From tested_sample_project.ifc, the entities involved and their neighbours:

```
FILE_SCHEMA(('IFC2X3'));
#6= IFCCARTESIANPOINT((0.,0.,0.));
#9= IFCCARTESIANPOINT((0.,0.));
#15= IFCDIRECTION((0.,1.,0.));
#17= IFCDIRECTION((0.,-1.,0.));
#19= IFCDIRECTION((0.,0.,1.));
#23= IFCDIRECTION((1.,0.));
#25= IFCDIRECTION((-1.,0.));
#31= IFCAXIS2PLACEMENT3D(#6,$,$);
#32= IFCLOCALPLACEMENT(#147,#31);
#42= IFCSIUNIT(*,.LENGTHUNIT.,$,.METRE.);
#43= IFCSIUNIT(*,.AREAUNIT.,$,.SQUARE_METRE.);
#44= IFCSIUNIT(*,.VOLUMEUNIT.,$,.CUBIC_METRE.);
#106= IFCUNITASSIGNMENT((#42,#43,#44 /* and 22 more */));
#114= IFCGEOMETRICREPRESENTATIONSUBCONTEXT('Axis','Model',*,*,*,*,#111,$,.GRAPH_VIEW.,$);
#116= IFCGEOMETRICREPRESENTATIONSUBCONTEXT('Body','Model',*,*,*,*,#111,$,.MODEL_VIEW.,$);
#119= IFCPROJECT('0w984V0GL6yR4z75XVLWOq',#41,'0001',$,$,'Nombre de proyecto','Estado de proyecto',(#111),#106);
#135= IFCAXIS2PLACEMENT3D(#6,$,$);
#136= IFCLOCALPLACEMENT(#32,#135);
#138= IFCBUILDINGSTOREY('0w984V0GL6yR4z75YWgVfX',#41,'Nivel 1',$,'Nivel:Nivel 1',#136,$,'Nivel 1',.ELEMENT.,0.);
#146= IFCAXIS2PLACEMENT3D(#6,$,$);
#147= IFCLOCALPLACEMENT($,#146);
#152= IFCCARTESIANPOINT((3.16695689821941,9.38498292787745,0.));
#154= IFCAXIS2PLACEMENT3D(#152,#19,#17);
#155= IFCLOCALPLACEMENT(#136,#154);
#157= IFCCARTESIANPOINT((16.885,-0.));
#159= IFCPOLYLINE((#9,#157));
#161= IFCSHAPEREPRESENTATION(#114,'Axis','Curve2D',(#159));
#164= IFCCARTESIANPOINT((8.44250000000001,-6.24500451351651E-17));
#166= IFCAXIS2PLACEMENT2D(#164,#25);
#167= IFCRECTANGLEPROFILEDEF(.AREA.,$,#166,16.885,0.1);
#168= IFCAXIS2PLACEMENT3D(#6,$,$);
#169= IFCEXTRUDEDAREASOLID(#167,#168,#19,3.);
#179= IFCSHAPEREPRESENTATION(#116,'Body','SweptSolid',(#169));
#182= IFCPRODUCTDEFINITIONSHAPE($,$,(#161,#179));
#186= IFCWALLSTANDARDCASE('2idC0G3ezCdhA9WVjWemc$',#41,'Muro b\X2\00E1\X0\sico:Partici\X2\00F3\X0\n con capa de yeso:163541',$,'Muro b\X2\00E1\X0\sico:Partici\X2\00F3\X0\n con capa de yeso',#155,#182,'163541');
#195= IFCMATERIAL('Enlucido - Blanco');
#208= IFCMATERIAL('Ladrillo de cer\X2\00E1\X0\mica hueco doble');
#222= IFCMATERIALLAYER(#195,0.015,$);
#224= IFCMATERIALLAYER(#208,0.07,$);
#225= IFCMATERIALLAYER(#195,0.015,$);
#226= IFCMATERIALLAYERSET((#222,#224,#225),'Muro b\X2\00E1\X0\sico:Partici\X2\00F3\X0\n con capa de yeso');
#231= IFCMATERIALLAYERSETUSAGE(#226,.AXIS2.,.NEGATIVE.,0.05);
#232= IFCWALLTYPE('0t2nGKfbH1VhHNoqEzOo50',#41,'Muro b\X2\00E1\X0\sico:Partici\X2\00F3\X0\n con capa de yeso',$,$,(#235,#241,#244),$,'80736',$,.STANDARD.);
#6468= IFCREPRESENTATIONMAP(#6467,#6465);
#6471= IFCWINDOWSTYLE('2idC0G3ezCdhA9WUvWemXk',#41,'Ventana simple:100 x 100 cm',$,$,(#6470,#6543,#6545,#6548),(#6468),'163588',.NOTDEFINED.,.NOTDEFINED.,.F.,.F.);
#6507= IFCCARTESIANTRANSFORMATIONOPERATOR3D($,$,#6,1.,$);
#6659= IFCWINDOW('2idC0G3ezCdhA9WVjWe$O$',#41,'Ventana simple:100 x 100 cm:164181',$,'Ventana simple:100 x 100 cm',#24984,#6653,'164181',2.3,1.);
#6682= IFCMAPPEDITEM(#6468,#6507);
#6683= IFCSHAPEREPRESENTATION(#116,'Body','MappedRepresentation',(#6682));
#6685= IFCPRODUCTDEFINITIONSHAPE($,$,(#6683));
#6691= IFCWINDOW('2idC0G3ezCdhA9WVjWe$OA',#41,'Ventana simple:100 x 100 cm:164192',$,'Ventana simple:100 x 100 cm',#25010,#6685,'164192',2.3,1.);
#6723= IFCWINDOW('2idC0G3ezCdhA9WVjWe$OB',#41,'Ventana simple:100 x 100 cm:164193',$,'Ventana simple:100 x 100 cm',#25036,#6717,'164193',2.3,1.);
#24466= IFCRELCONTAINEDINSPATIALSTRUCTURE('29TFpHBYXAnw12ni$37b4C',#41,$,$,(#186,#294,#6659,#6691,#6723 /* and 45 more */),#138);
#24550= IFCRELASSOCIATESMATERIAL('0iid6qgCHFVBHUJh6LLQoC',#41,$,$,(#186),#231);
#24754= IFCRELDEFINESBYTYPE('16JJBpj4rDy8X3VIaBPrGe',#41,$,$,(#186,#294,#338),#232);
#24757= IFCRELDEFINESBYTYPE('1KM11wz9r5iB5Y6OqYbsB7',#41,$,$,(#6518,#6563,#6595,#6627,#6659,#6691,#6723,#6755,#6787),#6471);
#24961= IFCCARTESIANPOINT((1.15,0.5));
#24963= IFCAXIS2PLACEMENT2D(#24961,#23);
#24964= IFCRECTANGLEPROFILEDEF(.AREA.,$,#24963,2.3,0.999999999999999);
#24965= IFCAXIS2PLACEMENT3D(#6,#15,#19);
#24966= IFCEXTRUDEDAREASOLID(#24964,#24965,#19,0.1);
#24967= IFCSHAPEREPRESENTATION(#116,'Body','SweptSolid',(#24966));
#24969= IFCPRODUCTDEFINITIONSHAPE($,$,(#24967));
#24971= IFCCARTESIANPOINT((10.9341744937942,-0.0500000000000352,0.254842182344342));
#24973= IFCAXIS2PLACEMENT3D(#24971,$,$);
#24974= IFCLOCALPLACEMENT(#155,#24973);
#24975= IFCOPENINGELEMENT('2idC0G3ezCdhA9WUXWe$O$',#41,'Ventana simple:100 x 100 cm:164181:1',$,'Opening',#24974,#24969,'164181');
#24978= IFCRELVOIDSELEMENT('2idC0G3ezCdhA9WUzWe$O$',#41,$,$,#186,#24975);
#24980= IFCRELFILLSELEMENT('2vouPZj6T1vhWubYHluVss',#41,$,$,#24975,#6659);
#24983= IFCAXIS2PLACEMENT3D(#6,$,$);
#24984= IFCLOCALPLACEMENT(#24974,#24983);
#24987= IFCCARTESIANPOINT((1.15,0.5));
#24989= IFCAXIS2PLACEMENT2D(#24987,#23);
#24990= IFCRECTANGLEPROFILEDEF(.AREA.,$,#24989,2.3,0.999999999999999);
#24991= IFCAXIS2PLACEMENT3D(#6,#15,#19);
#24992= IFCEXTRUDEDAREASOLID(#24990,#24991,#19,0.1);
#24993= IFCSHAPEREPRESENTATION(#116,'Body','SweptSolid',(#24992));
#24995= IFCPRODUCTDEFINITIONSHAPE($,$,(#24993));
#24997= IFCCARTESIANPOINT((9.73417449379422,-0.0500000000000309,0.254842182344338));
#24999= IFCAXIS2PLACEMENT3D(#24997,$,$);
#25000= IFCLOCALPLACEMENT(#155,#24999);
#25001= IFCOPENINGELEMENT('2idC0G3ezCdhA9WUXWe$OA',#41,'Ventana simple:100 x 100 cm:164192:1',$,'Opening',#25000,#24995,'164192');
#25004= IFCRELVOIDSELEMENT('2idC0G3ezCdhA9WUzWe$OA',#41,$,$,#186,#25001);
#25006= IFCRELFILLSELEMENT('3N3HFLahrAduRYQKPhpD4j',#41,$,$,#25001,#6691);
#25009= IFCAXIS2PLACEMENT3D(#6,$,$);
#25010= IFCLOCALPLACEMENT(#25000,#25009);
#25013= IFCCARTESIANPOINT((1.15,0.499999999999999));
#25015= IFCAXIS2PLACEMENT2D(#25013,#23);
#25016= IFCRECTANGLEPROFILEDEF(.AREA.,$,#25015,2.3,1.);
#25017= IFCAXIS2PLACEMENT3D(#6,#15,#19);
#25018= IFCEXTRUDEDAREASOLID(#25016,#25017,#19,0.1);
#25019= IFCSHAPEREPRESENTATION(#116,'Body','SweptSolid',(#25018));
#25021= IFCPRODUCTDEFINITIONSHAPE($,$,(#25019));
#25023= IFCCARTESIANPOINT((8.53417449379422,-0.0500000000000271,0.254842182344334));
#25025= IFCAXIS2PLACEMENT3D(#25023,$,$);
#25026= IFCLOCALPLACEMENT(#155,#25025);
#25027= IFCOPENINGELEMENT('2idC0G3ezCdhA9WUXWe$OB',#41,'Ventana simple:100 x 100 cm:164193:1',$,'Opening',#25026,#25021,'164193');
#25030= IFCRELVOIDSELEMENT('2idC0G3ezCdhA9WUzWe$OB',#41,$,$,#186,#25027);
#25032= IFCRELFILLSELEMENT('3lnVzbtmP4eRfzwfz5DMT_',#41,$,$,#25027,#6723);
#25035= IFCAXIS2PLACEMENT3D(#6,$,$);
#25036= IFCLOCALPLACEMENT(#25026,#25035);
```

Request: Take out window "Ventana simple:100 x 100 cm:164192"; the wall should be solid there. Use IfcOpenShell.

```python
import ifcopenshell
import ifcopenshell.api.feature
import ifcopenshell.api.root
import ifcopenshell.geom
import ifcopenshell.util.shape

model = ifcopenshell.open("tested_sample_project.ifc")
settings = ifcopenshell.geom.settings()


def volume(element):
    """Net volume in cubic metres, openings subtracted."""
    shape = ifcopenshell.geom.create_shape(settings, element)
    return ifcopenshell.util.shape.get_volume(shape.geometry)


window = model.by_guid("2idC0G3ezCdhA9WVjWe$OA")
opening = window.FillsVoids[0].RelatingOpeningElement
wall = opening.VoidsElements[0].RelatingBuildingElement
before = volume(wall)

ifcopenshell.api.root.remove_product(model, product=window)
ifcopenshell.api.feature.remove_feature(model, feature=opening)

after = volume(wall)

print(f"wall volume {before:.3f} -> {after:.3f} m3")

model.write("tested_sample_project_edited.ifc")
```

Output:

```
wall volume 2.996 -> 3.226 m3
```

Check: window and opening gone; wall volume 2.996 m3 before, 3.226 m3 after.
